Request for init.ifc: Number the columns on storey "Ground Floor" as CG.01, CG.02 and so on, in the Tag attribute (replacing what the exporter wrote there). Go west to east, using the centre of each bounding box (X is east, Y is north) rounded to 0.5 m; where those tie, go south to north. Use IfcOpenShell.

First a look at what the model holds.

```python
import ifcopenshell
import ifcopenshell.util.element
import ifcopenshell.util.placement

model = ifcopenshell.open("init.ifc")
print(model.schema)
storey = next(s for s in model.by_type("IfcBuildingStorey") if s.Name == "Ground Floor")
columns = [e for e in ifcopenshell.util.element.get_decomposition(storey) if e.is_a("IfcColumn")]
for e in sorted(columns, key=lambda e: e.id()):
    origin = ifcopenshell.util.placement.get_local_placement(e.ObjectPlacement)[:3, 3]
    print(e.id(), e.Tag, e.Name, origin.round(2) + 0.0, sep=" | ")
```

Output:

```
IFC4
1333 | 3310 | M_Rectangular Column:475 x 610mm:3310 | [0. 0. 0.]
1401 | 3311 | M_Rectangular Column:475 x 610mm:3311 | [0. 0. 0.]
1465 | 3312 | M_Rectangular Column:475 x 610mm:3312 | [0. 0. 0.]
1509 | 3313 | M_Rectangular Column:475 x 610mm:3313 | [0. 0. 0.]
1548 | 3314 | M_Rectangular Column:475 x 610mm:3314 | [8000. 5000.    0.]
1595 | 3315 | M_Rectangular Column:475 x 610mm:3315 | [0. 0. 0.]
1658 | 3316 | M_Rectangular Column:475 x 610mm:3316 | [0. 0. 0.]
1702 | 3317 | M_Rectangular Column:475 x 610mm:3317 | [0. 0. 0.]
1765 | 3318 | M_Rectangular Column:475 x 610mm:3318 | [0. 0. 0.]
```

```python
import ifcopenshell
import ifcopenshell.geom
import ifcopenshell.util.element
import ifcopenshell.util.shape

model = ifcopenshell.open("init.ifc")
settings = ifcopenshell.geom.settings()
settings.set("use-world-coords", True)


def centre(element):
    shape = ifcopenshell.geom.create_shape(settings, element)
    return ifcopenshell.util.shape.get_bbox_centroid(shape.geometry)


storey = next(s for s in model.by_type("IfcBuildingStorey") if s.Name == "Ground Floor")
columns = [e for e in ifcopenshell.util.element.get_decomposition(storey) if e.is_a("IfcColumn")]

# Insertion points can sit at a corner or the storey origin, so sort by the geometry (in metres).
centres = {e: centre(e) for e in columns}
columns.sort(key=lambda e: (round(centres[e][0] / 0.5), centres[e][1]))

for i, e in enumerate(columns, start=1):
    number = f"CG.{i:02d}"
    e.Tag = number
    print(e.id(), number)

model.write("init_edited.ifc")
```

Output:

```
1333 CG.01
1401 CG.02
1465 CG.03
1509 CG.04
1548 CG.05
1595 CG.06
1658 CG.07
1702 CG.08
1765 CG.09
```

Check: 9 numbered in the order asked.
